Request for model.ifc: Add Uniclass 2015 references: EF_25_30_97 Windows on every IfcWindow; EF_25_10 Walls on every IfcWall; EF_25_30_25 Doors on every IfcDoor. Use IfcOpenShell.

First a look at what the model holds.

```python
import ifcopenshell

model = ifcopenshell.open("model.ifc")
print(model.schema)
print("classifications:", [c.Name for c in model.by_type("IfcClassification")])
for ifc_class in ("IfcDoor", "IfcRoof", "IfcStair", "IfcWall", "IfcWindow"):
    print(ifc_class, len(model.by_type(ifc_class)))
```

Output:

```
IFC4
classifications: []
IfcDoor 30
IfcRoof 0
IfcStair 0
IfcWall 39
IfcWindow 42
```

```python
import ifcopenshell
import ifcopenshell.api.classification

model = ifcopenshell.open("model.ifc")

system = ifcopenshell.api.classification.add_classification(model, classification="Uniclass 2015")

codes = {
    "IfcWindow": ("EF_25_30_97", "Windows"),
    "IfcWall": ("EF_25_10", "Walls"),
    "IfcDoor": ("EF_25_30_25", "Doors"),
}
for ifc_class, (code, name) in codes.items():
    products = model.by_type(ifc_class)
    ifcopenshell.api.classification.add_reference(
        model, products=products, classification=system, identification=code, name=name
    )
    print(code, len(products))

model.write("model-out.ifc")
```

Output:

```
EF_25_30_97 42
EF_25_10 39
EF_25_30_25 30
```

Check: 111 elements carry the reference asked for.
